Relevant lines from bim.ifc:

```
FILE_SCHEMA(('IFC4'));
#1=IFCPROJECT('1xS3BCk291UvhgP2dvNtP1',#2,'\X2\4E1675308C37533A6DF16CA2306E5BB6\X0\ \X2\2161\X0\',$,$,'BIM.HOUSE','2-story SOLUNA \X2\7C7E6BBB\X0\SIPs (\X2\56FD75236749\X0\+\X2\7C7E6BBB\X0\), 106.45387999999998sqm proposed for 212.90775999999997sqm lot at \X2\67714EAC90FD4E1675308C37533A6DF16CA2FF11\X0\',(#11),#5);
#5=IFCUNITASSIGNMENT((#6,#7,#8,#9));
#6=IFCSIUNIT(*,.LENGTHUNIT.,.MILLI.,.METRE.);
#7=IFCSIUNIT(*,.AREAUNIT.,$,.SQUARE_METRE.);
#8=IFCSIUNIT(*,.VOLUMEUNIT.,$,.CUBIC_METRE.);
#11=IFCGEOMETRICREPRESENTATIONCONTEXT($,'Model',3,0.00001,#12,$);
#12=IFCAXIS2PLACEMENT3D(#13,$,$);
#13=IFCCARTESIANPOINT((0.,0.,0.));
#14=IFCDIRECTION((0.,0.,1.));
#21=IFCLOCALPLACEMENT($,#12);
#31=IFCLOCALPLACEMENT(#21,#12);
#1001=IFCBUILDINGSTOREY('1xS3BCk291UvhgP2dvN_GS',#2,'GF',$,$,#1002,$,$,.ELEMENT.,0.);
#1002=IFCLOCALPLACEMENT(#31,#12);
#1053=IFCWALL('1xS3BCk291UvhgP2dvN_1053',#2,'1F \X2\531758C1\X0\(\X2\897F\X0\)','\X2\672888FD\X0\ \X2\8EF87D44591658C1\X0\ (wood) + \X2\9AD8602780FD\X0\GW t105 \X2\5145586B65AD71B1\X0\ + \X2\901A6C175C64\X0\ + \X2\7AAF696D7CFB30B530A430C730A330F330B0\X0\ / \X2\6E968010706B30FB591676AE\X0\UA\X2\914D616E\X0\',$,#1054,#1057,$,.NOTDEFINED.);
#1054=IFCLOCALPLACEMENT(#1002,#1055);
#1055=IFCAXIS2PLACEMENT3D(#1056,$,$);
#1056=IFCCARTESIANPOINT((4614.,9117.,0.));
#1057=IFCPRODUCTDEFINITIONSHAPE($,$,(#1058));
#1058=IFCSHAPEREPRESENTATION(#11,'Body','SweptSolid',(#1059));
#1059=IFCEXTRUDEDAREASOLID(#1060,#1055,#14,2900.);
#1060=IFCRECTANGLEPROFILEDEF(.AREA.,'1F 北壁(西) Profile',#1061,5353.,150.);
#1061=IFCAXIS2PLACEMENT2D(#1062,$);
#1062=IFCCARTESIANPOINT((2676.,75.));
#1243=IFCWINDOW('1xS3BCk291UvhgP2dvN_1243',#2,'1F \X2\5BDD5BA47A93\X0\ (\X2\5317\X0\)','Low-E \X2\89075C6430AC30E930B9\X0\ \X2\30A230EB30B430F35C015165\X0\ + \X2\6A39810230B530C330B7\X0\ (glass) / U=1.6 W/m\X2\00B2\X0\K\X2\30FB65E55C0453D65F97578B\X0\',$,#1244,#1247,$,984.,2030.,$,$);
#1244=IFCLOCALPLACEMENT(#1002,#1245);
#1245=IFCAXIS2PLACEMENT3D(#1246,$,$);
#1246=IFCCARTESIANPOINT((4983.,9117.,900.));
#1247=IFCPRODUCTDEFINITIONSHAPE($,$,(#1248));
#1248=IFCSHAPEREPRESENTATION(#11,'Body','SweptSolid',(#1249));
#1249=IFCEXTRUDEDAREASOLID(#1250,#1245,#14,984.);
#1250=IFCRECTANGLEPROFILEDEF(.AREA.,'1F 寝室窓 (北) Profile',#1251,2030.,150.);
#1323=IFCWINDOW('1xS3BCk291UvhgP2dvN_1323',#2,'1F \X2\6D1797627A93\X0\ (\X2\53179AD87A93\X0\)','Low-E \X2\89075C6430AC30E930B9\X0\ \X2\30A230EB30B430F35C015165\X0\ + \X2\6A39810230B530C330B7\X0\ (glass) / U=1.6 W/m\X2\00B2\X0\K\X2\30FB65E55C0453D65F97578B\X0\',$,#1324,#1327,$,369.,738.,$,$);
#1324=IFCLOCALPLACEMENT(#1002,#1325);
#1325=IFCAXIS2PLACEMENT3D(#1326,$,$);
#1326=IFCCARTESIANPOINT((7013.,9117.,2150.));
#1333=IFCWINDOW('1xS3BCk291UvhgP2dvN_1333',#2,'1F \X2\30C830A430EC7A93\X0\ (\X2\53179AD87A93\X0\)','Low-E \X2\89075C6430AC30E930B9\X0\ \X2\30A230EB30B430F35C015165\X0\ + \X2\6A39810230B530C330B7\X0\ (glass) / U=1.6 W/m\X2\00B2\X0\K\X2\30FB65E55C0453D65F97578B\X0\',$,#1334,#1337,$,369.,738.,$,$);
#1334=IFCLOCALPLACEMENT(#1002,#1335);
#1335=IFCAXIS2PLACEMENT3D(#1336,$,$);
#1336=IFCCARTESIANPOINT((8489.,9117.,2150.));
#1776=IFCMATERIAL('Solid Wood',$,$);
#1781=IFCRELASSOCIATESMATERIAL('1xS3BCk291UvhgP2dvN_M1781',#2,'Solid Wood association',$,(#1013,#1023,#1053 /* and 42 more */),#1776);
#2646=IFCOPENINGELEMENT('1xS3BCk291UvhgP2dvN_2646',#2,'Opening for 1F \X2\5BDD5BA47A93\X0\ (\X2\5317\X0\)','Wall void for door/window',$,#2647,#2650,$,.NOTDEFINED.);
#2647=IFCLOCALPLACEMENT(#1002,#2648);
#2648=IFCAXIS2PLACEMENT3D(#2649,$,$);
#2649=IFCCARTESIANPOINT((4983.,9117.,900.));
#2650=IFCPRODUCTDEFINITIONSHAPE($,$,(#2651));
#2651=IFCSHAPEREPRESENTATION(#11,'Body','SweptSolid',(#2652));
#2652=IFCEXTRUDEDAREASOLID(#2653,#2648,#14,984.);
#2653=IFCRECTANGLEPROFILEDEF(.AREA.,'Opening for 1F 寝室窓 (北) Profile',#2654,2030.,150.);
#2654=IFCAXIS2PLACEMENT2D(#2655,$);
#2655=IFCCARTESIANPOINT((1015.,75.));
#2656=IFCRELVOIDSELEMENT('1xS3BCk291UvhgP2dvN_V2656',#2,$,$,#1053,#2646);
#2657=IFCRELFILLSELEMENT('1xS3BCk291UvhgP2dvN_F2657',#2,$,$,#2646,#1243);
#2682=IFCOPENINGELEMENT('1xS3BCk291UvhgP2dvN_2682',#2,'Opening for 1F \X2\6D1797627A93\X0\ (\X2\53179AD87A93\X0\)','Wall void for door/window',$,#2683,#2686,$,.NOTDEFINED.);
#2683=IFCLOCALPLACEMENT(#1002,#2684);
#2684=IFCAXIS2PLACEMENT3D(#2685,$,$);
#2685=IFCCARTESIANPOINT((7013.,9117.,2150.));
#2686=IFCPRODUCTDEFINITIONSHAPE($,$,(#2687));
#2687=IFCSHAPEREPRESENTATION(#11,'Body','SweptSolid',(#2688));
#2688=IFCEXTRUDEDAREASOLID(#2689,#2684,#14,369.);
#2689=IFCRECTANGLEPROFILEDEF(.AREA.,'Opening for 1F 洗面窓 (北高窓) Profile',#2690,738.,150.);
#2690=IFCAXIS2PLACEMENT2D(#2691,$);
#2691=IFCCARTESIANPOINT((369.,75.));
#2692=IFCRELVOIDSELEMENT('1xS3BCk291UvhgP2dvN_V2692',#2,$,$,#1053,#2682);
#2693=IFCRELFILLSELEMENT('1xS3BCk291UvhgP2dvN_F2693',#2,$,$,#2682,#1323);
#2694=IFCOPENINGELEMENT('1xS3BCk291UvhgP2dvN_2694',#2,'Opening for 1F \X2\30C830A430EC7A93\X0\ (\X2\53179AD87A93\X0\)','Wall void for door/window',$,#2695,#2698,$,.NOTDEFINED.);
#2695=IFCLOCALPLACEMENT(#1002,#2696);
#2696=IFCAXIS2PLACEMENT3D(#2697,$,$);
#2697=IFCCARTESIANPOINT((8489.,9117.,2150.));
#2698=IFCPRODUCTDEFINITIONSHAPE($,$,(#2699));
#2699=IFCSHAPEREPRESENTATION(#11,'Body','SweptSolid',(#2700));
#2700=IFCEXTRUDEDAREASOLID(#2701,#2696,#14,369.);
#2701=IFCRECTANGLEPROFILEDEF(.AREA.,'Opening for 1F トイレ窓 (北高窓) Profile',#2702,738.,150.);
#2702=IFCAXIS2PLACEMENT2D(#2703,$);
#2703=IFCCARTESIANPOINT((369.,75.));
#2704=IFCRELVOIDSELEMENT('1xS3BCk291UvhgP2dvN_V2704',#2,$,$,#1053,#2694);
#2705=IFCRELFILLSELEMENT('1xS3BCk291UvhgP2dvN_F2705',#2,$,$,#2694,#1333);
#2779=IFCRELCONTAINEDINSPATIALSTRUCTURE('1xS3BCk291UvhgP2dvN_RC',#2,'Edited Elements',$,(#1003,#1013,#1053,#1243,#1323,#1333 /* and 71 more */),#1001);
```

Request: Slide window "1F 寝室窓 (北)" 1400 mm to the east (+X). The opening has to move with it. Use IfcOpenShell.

```python
import ifcopenshell
import ifcopenshell.api.geometry
import ifcopenshell.util.placement
import ifcopenshell.util.unit

model = ifcopenshell.open("bim.ifc")
unit_scale = ifcopenshell.util.unit.calculate_unit_scale(model)

window = model.by_guid("1xS3BCk291UvhgP2dvN_1243")
opening = window.FillsVoids[0].RelatingOpeningElement
wall = opening.VoidsElements[0].RelatingBuildingElement

wall_matrix = ifcopenshell.util.placement.get_local_placement(wall.ObjectPlacement)
shift = wall_matrix[:3, 0] * 1.4 / unit_scale
before = ifcopenshell.util.placement.get_local_placement(window.ObjectPlacement)[:3, 3].copy()

# The window is not placed relative to its opening, so move both.
for product in (opening, window):
    matrix = ifcopenshell.util.placement.get_local_placement(product.ObjectPlacement)
    matrix[:3, 3] += shift
    ifcopenshell.api.geometry.edit_object_placement(model, product=product, matrix=matrix, is_si=False)

after = ifcopenshell.util.placement.get_local_placement(window.ObjectPlacement)[:3, 3]
print("window moved by", (after - before).round(3) + 0.0)

model.write("bim_updated.ifc")
```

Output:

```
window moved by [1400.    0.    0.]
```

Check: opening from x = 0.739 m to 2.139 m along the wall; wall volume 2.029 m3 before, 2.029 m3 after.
